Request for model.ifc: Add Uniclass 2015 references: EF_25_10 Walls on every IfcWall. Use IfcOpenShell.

First a look at what the model holds.

```python
import ifcopenshell

model = ifcopenshell.open("model.ifc")
print(model.schema)
print("classifications:", [c.Name for c in model.by_type("IfcClassification")])
for ifc_class in ("IfcDoor", "IfcRoof", "IfcStair", "IfcWall", "IfcWindow"):
    print(ifc_class, len(model.by_type(ifc_class)))
```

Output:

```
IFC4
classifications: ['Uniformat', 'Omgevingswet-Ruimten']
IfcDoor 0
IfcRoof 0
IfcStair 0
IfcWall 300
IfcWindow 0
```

```python
import ifcopenshell
import ifcopenshell.api.classification

model = ifcopenshell.open("model.ifc")

system = ifcopenshell.api.classification.add_classification(model, classification="Uniclass 2015")

codes = {
    "IfcWall": ("EF_25_10", "Walls"),
}
for ifc_class, (code, name) in codes.items():
    products = model.by_type(ifc_class)
    ifcopenshell.api.classification.add_reference(
        model, products=products, classification=system, identification=code, name=name
    )
    print(code, len(products))

model.write("model_rev.ifc")
```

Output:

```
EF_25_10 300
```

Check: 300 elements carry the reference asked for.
